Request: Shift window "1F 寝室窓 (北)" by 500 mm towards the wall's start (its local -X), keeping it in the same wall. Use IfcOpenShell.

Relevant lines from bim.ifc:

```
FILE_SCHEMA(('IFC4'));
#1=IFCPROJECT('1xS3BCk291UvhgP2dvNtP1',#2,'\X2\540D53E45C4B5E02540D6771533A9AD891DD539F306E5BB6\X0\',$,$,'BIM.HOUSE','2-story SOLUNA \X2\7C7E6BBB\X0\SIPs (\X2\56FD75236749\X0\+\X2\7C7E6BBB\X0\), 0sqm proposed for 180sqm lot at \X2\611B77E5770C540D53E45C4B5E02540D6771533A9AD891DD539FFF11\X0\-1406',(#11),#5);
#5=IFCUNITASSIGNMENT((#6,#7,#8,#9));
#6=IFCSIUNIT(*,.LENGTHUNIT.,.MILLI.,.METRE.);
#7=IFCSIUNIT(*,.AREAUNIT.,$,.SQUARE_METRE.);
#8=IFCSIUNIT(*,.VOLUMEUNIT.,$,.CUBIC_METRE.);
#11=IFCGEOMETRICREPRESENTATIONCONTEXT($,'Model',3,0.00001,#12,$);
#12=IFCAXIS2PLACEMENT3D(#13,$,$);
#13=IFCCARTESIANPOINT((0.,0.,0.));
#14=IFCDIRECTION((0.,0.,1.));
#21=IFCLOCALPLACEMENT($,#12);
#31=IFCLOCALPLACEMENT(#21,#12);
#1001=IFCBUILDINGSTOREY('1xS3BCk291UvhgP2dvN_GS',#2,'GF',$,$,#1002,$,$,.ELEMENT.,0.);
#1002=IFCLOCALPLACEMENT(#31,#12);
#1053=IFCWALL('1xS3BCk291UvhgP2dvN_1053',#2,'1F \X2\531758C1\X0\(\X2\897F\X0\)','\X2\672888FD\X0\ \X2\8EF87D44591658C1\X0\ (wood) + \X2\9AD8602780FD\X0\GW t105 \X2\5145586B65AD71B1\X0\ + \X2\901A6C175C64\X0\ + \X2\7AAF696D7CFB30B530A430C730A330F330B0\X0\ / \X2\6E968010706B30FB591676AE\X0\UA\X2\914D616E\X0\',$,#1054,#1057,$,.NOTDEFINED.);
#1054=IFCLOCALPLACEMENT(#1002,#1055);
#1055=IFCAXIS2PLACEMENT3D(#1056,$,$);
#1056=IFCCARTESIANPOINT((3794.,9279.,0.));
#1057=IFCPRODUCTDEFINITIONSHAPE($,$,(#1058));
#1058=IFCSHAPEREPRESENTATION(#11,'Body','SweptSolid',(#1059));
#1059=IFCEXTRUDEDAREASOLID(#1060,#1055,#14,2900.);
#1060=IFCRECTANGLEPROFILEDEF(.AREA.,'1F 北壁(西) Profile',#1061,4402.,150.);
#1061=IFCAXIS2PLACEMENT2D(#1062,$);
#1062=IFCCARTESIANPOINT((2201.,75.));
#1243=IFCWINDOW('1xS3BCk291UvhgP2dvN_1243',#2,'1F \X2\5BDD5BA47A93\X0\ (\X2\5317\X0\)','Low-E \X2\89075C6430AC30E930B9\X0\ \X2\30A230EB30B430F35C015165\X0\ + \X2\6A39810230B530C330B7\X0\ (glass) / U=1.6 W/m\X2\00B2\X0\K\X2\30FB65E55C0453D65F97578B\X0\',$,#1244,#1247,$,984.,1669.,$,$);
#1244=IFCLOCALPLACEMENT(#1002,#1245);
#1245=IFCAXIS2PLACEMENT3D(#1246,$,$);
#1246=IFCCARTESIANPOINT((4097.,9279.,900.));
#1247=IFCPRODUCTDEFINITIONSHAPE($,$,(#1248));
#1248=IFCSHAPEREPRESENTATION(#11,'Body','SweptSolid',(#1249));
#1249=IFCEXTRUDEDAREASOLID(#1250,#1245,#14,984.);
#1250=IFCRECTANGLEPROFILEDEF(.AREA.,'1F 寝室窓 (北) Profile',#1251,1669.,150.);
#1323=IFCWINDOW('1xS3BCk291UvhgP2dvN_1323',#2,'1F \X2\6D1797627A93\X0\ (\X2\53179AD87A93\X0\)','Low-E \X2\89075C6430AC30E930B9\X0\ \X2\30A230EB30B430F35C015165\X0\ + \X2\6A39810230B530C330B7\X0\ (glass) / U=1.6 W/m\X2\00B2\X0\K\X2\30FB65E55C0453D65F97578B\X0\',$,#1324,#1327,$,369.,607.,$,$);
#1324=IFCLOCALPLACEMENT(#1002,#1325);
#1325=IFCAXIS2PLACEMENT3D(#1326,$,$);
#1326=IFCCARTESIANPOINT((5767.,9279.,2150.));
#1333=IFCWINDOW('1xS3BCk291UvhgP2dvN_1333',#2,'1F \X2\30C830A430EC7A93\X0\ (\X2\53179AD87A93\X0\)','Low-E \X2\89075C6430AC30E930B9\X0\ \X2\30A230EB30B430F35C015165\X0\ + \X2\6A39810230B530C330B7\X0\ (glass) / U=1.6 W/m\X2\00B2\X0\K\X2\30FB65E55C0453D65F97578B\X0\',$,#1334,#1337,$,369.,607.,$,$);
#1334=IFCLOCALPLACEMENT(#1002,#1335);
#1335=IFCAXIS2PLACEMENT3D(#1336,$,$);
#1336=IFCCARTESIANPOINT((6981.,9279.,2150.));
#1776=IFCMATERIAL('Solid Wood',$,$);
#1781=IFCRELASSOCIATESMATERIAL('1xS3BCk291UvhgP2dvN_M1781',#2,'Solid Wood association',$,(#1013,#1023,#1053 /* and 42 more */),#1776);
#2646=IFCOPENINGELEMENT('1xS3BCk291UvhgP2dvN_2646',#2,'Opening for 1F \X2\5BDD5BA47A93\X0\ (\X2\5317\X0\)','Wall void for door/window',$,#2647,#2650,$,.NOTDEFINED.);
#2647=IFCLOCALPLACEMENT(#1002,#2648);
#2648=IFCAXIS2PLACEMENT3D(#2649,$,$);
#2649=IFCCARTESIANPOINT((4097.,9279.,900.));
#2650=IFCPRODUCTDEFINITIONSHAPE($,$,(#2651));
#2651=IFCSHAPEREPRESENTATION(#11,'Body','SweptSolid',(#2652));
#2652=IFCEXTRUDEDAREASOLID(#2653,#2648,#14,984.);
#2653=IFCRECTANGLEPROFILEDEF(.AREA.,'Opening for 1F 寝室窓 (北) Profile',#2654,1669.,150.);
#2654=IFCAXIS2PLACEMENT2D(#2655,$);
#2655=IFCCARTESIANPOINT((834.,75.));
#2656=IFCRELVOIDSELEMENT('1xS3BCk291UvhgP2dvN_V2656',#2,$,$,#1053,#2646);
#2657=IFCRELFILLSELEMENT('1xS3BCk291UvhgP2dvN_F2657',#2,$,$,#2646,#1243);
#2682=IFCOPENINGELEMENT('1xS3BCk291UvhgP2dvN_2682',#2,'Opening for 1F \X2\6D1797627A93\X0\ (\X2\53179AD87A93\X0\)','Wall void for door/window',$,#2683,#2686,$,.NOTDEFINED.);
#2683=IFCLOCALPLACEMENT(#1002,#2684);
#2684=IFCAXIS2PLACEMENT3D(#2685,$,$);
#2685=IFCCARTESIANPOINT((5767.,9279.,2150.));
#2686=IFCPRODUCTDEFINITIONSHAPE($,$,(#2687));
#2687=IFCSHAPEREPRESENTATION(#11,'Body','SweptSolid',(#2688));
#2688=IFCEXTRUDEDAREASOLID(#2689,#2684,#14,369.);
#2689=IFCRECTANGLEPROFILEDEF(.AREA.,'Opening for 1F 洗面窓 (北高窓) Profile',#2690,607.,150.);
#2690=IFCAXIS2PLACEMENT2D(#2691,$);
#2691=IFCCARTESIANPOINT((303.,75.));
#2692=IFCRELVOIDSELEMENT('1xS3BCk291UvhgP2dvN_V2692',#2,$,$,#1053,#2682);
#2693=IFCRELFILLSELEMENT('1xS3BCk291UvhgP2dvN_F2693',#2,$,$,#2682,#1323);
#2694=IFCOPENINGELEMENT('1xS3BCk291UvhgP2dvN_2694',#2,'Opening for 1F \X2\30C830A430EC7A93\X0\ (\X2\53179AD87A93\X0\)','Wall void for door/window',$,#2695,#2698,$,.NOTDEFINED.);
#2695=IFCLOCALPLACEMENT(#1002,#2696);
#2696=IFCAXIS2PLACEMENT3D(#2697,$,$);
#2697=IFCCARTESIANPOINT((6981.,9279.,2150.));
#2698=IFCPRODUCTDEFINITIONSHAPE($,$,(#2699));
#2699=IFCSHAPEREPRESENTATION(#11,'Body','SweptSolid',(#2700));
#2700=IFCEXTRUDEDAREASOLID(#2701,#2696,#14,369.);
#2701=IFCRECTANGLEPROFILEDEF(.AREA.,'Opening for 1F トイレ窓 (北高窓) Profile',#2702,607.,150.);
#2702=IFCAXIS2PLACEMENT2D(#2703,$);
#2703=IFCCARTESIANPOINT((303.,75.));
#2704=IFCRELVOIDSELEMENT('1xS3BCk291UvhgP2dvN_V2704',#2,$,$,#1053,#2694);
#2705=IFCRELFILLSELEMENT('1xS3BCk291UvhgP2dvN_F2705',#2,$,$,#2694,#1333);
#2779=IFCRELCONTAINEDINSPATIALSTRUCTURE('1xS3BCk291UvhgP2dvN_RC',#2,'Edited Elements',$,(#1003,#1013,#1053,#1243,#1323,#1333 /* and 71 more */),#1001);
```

```python
import ifcopenshell
import ifcopenshell.api.geometry
import ifcopenshell.util.placement

model = ifcopenshell.open("bim.ifc")

window = model.by_id(1243)
opening = window.FillsVoids[0].RelatingOpeningElement
wall = opening.VoidsElements[0].RelatingBuildingElement

wall_matrix = ifcopenshell.util.placement.get_local_placement(wall.ObjectPlacement)
shift = wall_matrix[:3, 0] * -500.0
before = ifcopenshell.util.placement.get_local_placement(window.ObjectPlacement)[:3, 3].copy()

# The window is not placed relative to its opening, so move both.
for product in (opening, window):
    matrix = ifcopenshell.util.placement.get_local_placement(product.ObjectPlacement)
    matrix[:3, 3] += shift
    ifcopenshell.api.geometry.edit_object_placement(model, product=product, matrix=matrix, is_si=False)

after = ifcopenshell.util.placement.get_local_placement(window.ObjectPlacement)[:3, 3]
print("window moved by", (after - before).round(3) + 0.0)

model.write("bim_rev.ifc")
```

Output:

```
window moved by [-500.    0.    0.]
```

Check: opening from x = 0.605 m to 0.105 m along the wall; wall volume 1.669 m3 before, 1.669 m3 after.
